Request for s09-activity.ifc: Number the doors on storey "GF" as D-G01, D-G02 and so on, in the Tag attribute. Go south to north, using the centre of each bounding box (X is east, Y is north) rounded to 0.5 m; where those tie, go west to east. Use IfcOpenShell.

First a look at what the model holds.

```python
import ifcopenshell
import ifcopenshell.util.element
import ifcopenshell.util.placement

model = ifcopenshell.open("s09-activity.ifc")
print(model.schema)
storey = next(s for s in model.by_type("IfcBuildingStorey") if s.Name == "GF")
doors = [e for e in ifcopenshell.util.element.get_decomposition(storey) if e.is_a("IfcDoor")]
for e in sorted(doors, key=lambda e: e.id()):
    origin = ifcopenshell.util.placement.get_local_placement(e.ObjectPlacement)[:3, 3]
    print(e.id(), e.Tag, e.Name, origin.round(2) + 0.0, sep=" | ")
```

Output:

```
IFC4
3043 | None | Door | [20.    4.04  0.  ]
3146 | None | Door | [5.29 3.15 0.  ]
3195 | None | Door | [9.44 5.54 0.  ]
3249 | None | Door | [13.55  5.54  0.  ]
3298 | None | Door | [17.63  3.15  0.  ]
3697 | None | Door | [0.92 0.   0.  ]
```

```python
import ifcopenshell
import ifcopenshell.geom
import ifcopenshell.util.element
import ifcopenshell.util.shape

model = ifcopenshell.open("s09-activity.ifc")
settings = ifcopenshell.geom.settings()
settings.set("use-world-coords", True)


def centre(element):
    shape = ifcopenshell.geom.create_shape(settings, element)
    return ifcopenshell.util.shape.get_bbox_centroid(shape.geometry)


storey = next(s for s in model.by_type("IfcBuildingStorey") if s.Name == "GF")
doors = [e for e in ifcopenshell.util.element.get_decomposition(storey) if e.is_a("IfcDoor")]

# Insertion points can sit at a corner or the storey origin, so sort by the geometry (in metres).
centres = {e: centre(e) for e in doors}
doors.sort(key=lambda e: (round(centres[e][1] / 0.5), centres[e][0]))

for i, e in enumerate(doors, start=1):
    number = f"D-G{i:02d}"
    e.Tag = number
    print(e.id(), number)

model.write("s09-activity_edited.ifc")
```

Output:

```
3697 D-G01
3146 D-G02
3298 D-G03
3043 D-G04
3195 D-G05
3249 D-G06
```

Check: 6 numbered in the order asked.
